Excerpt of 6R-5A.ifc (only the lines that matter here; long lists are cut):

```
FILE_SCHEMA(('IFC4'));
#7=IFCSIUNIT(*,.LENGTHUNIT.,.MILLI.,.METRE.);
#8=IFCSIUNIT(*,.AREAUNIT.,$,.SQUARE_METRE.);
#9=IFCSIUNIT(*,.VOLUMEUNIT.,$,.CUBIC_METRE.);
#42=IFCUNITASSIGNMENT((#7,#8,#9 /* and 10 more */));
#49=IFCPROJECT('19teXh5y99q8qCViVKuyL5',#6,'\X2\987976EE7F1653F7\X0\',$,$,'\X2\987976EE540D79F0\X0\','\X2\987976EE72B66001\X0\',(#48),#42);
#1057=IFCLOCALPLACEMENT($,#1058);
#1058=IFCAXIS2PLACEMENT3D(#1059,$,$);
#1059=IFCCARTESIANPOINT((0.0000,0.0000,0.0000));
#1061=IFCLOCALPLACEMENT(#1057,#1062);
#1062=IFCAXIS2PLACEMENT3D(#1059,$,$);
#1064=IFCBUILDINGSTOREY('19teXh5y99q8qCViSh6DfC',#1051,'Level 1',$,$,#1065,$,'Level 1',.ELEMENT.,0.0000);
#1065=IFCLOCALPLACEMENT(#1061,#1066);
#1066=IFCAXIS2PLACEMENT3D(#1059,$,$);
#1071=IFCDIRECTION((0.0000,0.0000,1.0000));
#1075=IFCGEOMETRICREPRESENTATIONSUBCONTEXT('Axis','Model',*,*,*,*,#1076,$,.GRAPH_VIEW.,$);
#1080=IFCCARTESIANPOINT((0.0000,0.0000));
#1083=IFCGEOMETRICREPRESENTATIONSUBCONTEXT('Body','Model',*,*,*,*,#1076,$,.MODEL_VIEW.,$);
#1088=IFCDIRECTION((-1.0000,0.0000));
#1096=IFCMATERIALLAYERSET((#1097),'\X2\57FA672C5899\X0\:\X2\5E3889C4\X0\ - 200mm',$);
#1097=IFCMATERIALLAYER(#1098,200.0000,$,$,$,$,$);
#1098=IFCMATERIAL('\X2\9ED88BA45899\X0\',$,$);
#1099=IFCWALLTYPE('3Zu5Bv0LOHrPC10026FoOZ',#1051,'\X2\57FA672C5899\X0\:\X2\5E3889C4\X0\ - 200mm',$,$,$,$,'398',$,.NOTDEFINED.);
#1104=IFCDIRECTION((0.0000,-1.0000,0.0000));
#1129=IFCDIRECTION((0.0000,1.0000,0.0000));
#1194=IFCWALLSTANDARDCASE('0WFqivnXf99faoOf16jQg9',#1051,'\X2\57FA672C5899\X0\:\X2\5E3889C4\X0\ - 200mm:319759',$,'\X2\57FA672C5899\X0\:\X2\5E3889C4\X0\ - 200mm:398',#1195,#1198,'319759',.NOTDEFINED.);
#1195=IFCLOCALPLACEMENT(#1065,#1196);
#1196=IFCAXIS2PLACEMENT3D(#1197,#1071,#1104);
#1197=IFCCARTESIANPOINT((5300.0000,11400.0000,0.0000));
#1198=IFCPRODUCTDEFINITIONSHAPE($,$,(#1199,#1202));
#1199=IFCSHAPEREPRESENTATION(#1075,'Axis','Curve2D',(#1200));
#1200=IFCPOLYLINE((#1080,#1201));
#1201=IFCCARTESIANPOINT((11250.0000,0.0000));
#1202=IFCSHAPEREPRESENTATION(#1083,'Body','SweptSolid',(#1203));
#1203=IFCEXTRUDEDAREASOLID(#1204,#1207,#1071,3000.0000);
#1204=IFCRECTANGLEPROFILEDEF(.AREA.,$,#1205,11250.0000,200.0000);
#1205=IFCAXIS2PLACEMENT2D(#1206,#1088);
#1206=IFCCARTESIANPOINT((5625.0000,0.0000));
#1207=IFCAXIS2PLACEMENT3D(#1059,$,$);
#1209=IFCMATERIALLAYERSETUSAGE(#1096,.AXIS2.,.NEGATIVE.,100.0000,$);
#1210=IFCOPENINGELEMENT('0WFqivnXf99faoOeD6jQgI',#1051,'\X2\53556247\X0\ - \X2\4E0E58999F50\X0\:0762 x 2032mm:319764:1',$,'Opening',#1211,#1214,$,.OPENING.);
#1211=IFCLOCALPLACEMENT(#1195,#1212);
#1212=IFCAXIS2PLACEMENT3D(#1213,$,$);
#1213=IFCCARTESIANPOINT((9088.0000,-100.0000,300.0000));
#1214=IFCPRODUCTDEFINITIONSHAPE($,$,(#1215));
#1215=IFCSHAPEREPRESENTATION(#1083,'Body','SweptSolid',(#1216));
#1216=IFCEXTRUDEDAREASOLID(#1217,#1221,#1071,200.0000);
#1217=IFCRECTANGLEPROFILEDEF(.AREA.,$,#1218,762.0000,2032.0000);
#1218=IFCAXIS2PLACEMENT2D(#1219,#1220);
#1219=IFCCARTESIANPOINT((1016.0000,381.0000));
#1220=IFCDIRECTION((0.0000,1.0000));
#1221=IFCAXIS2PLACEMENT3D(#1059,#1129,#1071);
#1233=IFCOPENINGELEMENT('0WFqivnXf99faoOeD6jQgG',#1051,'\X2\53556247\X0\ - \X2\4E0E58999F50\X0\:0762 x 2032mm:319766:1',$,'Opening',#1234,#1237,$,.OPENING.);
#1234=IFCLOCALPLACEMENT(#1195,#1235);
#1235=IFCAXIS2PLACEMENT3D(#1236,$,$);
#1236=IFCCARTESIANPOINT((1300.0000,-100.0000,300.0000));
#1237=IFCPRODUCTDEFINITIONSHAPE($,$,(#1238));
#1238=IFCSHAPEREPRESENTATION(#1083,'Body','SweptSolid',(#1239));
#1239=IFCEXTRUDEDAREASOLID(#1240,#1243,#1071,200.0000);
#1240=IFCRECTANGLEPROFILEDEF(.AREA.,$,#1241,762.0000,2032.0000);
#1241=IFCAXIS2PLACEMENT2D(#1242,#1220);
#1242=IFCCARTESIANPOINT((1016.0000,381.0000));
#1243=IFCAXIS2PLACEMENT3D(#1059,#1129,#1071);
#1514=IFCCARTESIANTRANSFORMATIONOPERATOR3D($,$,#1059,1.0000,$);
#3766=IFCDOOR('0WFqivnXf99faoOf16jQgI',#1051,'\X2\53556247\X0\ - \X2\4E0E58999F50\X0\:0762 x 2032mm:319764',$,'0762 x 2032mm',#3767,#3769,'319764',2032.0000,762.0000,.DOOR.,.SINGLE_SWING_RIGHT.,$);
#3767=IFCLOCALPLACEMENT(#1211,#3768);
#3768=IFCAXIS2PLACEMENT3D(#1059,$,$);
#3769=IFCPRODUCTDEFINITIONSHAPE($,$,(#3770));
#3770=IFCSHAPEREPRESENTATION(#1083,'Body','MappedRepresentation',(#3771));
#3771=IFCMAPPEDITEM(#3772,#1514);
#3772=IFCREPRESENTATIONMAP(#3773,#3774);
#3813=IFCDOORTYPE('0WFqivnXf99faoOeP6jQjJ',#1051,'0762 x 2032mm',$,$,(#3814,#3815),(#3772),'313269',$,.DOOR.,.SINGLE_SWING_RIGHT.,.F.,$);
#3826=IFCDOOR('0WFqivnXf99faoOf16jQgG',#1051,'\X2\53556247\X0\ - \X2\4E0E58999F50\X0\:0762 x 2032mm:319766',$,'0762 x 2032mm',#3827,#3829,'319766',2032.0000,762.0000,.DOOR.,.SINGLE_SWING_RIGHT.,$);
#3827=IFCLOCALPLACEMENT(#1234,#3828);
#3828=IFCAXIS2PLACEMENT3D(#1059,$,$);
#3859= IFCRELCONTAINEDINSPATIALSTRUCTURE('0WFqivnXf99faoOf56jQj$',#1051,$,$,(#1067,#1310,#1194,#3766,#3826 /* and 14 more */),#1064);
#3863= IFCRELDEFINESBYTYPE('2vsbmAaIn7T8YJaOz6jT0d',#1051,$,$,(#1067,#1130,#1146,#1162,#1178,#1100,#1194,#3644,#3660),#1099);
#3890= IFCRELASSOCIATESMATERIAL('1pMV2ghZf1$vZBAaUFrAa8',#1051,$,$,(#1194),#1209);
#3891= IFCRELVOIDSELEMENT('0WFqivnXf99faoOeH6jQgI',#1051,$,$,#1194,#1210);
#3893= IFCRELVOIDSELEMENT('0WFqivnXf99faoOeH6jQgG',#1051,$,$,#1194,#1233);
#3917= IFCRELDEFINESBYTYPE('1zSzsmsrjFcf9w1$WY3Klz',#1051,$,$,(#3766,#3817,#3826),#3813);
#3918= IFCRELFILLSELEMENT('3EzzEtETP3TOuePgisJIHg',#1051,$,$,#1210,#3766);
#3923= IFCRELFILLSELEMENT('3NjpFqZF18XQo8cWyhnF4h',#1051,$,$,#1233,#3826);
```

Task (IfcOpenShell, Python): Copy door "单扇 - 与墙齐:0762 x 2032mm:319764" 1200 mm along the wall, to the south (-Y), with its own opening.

```python
import ifcopenshell
import ifcopenshell.api.feature
import ifcopenshell.api.geometry
import ifcopenshell.api.root
import ifcopenshell.geom
import ifcopenshell.util.element
import ifcopenshell.util.placement
import ifcopenshell.util.shape

model = ifcopenshell.open("6R-5A.ifc")
settings = ifcopenshell.geom.settings()


def volume(element):
    """Net volume in cubic metres, openings subtracted."""
    shape = ifcopenshell.geom.create_shape(settings, element)
    return ifcopenshell.util.shape.get_volume(shape.geometry)


def reuse_history(source, copy):
    """copy_class also copies each property set's owner history, people and application; keep the originals."""
    for rel in copy.IsDefinedBy:
        if rel.is_a("IfcRelDefinesByProperties") and (history := rel.RelatingPropertyDefinition.OwnerHistory):
            rel.RelatingPropertyDefinition.OwnerHistory = source.OwnerHistory
            ifcopenshell.util.element.remove_deep2(model, history)


door = model.by_guid("0WFqivnXf99faoOf16jQgI")
opening = door.FillsVoids[0].RelatingOpeningElement
wall = opening.VoidsElements[0].RelatingBuildingElement
before = volume(wall)
shift = ifcopenshell.util.placement.get_local_placement(wall.ObjectPlacement)[:3, 0] * 1200.0

# copy_class copies the void relationship, type, container and properties, but no geometry.
new_opening = ifcopenshell.api.root.copy_class(model, product=opening)
new_opening.Representation = ifcopenshell.util.element.copy_deep(
    model, opening.Representation, exclude=["IfcGeometricRepresentationContext", "IfcRepresentationMap"]
)
new_opening.Name = "单扇 - 与墙齐:0762 x 2032mm"
new_door = ifcopenshell.api.root.copy_class(model, product=door)
new_door.Representation = ifcopenshell.util.element.copy_deep(
    model, door.Representation, exclude=["IfcGeometricRepresentationContext", "IfcRepresentationMap"]
)
new_door.Name = "单扇 - 与墙齐:0762 x 2032mm"
new_door.Tag = None
reuse_history(door, new_door)
ifcopenshell.api.feature.add_filling(model, opening=new_opening, element=new_door)

for old, new in ((opening, new_opening), (door, new_door)):
    matrix = ifcopenshell.util.placement.get_local_placement(old.ObjectPlacement)
    matrix[:3, 3] += shift
    ifcopenshell.api.geometry.edit_object_placement(model, product=new, matrix=matrix, is_si=False)

after = volume(wall)

print(f"wall volume {before:.3f} -> {after:.3f} m3")

model.write("6R-5A_rev.ifc")
```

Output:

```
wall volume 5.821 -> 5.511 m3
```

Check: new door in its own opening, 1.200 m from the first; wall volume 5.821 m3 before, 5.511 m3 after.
